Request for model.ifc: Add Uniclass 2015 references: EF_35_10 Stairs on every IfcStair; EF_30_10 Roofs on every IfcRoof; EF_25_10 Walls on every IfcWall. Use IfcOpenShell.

First a look at what the model holds.

```python
import ifcopenshell

model = ifcopenshell.open("model.ifc")
print(model.schema)
print("classifications:", [c.Name for c in model.by_type("IfcClassification")])
for ifc_class in ("IfcDoor", "IfcRoof", "IfcStair", "IfcWall", "IfcWindow"):
    print(ifc_class, len(model.by_type(ifc_class)))
```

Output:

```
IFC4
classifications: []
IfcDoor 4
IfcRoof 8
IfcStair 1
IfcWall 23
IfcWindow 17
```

```python
import ifcopenshell
import ifcopenshell.api.classification

model = ifcopenshell.open("model.ifc")

system = ifcopenshell.api.classification.add_classification(model, classification="Uniclass 2015")

codes = {
    "IfcStair": ("EF_35_10", "Stairs"),
    "IfcRoof": ("EF_30_10", "Roofs"),
    "IfcWall": ("EF_25_10", "Walls"),
}
for ifc_class, (code, name) in codes.items():
    products = model.by_type(ifc_class)
    ifcopenshell.api.classification.add_reference(
        model, products=products, classification=system, identification=code, name=name
    )
    print(code, len(products))

model.write("model_edited.ifc")
```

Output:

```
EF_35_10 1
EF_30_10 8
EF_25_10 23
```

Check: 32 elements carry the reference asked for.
